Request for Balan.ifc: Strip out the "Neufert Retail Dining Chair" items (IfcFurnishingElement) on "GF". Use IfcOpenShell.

First a look at what the model holds.

```python
import ifcopenshell
import ifcopenshell.util.element

model = ifcopenshell.open("Balan.ifc")
print(model.schema)
storey = next(s for s in model.by_type("IfcBuildingStorey") if s.Name == "GF")
furniture = [e for e in ifcopenshell.util.element.get_decomposition(storey) if e.is_a("IfcFurnishingElement")]
seen = {}
for e in furniture:
    element_type = ifcopenshell.util.element.get_type(e)
    name = element_type.Name if element_type not in (None, e) else None
    seen[name] = seen.get(name, 0) + 1
for name, count in sorted(seen.items(), key=str):
    print(count, "x", name)
```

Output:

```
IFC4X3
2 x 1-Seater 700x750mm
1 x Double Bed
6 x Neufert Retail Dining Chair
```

```python
import ifcopenshell
import ifcopenshell.api.root
import ifcopenshell.util.element

model = ifcopenshell.open("Balan.ifc")

storey = next(s for s in model.by_type("IfcBuildingStorey") if s.Name == "GF")
furniture = [e for e in ifcopenshell.util.element.get_decomposition(storey) if e.is_a("IfcFurnishingElement")]
targets = [e for e in furniture if (t := ifcopenshell.util.element.get_type(e)) not in (None, e) and t.Name == "Neufert Retail Dining Chair"]

for e in targets:
    ifcopenshell.api.root.remove_product(model, product=e)
print(len(targets), "removed")

model.write("Balan_v2.ifc")
```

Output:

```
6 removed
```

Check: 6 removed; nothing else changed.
